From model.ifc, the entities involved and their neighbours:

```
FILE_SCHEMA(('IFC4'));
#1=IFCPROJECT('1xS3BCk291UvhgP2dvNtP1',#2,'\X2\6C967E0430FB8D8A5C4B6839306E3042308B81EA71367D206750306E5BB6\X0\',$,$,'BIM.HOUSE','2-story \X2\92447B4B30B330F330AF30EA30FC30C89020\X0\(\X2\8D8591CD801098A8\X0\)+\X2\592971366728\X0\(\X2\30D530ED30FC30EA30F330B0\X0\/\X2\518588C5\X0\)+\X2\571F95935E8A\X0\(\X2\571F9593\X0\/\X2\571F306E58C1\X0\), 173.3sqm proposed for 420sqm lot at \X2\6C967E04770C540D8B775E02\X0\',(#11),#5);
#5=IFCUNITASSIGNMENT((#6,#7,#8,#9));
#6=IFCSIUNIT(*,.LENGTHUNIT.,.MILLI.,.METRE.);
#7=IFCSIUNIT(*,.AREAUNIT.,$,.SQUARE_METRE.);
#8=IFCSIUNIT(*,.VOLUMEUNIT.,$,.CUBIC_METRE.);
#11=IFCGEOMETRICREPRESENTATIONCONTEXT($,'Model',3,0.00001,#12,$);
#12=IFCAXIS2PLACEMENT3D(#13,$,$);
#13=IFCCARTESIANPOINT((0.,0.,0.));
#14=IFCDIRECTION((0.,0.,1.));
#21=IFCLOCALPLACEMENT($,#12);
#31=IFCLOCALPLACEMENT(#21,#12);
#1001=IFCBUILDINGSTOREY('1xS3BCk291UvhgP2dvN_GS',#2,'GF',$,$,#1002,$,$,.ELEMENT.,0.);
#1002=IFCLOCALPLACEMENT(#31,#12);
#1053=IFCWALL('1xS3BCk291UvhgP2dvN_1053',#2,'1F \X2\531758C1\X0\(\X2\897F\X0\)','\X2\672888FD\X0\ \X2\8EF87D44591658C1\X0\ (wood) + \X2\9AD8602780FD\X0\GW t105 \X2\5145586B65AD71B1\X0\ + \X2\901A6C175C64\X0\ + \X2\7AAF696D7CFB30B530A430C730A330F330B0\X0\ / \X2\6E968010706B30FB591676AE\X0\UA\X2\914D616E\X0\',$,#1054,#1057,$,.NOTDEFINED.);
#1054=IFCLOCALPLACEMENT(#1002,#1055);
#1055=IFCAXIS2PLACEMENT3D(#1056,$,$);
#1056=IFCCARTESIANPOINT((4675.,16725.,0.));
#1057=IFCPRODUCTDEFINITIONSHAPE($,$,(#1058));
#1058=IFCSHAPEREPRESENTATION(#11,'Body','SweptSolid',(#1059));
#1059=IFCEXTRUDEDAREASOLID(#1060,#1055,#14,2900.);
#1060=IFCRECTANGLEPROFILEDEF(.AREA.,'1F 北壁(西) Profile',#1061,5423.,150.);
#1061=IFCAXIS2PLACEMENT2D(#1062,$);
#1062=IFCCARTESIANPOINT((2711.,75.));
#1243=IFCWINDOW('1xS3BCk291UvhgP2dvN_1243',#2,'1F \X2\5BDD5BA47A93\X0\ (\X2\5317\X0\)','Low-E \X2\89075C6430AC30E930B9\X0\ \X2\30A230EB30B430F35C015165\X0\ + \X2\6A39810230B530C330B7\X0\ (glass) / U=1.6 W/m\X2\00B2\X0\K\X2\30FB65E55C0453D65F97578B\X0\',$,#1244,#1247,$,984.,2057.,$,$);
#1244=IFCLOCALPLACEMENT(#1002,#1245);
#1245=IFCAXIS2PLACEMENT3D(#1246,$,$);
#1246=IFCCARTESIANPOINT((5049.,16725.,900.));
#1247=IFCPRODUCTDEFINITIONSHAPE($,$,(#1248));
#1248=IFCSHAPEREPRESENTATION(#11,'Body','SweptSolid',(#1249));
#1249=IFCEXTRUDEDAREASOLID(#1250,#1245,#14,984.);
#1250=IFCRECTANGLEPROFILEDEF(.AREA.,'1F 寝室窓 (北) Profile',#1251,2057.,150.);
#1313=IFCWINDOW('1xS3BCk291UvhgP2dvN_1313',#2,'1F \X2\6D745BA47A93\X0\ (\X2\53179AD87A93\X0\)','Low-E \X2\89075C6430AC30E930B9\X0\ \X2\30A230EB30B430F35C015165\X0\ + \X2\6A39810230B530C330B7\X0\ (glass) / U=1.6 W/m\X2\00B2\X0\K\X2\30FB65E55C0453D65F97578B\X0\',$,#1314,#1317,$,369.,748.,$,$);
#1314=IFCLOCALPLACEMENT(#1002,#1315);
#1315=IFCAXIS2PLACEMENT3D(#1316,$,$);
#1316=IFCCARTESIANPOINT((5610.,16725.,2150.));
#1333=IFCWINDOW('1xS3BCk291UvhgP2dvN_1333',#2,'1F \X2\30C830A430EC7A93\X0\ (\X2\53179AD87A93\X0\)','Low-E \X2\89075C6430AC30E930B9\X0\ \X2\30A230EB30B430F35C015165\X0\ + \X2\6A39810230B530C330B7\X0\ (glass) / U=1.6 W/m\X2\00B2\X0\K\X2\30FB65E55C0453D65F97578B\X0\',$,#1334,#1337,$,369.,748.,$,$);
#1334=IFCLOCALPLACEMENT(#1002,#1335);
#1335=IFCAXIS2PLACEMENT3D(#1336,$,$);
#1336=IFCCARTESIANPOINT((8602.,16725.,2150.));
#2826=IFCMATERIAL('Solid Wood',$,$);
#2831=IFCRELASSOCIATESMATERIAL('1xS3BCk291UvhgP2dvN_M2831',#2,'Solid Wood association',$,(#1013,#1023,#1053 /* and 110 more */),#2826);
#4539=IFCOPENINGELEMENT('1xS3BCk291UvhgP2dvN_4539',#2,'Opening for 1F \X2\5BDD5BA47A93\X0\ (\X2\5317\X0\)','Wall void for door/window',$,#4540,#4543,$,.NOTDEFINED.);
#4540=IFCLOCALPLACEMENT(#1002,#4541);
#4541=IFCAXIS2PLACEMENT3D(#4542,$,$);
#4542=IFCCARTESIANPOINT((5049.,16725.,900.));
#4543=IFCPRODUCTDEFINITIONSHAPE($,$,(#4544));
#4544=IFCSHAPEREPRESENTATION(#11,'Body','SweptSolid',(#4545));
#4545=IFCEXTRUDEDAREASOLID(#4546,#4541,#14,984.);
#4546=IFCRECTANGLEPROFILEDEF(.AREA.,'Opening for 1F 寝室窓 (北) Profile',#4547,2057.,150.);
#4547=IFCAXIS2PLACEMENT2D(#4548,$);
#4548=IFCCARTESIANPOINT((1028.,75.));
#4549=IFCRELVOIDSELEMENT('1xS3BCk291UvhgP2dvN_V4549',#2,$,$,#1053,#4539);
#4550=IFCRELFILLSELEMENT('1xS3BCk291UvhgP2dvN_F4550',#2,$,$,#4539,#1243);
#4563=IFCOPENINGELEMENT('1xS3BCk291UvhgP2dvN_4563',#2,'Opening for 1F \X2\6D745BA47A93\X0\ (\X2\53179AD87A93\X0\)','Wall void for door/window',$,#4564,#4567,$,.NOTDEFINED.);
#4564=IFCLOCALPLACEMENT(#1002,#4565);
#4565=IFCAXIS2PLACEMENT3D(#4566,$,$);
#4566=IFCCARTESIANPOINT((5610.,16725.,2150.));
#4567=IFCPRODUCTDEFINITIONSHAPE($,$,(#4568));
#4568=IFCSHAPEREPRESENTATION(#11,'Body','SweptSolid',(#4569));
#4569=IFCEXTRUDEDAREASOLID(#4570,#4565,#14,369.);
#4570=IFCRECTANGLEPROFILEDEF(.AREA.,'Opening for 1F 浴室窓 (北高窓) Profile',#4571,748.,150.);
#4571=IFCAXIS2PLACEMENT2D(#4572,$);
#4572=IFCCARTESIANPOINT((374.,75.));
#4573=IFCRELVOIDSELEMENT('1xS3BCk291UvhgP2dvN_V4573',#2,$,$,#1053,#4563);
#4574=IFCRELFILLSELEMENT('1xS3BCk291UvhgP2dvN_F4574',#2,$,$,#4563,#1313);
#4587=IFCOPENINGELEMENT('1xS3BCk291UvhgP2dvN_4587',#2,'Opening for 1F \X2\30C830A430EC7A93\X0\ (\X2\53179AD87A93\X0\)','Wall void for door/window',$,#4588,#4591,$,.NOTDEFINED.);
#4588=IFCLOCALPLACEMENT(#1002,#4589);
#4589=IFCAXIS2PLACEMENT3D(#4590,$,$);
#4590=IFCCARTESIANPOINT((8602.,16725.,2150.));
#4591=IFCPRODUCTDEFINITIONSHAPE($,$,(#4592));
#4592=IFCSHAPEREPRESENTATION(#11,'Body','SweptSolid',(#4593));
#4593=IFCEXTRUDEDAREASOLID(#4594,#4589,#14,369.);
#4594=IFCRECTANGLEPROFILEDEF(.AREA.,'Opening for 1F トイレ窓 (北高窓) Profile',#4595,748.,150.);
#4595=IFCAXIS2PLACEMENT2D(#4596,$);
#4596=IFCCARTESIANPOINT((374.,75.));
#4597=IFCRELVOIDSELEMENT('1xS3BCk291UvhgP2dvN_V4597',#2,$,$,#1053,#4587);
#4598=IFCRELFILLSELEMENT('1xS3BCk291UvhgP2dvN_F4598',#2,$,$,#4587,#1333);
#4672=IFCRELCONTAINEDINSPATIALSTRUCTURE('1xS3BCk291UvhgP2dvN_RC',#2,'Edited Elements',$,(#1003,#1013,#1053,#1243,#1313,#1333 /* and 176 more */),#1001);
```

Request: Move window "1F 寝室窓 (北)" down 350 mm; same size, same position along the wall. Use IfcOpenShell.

```python
import numpy as np
import ifcopenshell
import ifcopenshell.api.geometry
import ifcopenshell.util.placement
import ifcopenshell.util.unit

model = ifcopenshell.open("model.ifc")
unit_scale = ifcopenshell.util.unit.calculate_unit_scale(model)

window = model.by_guid("1xS3BCk291UvhgP2dvN_1243")
opening = window.FillsVoids[0].RelatingOpeningElement
dz = -0.35 / unit_scale

shift = np.array([0.0, 0.0, dz])
# The window is not placed relative to its opening, so move both.
for product in (opening, window):
    matrix = ifcopenshell.util.placement.get_local_placement(product.ObjectPlacement)
    matrix[:3, 3] += shift
    ifcopenshell.api.geometry.edit_object_placement(model, product=product, matrix=matrix, is_si=False)

print(f"moved by {dz * unit_scale:+.3f} m")

model.write("model-out.ifc")
```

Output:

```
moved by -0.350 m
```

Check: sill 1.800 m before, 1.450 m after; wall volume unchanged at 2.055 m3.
